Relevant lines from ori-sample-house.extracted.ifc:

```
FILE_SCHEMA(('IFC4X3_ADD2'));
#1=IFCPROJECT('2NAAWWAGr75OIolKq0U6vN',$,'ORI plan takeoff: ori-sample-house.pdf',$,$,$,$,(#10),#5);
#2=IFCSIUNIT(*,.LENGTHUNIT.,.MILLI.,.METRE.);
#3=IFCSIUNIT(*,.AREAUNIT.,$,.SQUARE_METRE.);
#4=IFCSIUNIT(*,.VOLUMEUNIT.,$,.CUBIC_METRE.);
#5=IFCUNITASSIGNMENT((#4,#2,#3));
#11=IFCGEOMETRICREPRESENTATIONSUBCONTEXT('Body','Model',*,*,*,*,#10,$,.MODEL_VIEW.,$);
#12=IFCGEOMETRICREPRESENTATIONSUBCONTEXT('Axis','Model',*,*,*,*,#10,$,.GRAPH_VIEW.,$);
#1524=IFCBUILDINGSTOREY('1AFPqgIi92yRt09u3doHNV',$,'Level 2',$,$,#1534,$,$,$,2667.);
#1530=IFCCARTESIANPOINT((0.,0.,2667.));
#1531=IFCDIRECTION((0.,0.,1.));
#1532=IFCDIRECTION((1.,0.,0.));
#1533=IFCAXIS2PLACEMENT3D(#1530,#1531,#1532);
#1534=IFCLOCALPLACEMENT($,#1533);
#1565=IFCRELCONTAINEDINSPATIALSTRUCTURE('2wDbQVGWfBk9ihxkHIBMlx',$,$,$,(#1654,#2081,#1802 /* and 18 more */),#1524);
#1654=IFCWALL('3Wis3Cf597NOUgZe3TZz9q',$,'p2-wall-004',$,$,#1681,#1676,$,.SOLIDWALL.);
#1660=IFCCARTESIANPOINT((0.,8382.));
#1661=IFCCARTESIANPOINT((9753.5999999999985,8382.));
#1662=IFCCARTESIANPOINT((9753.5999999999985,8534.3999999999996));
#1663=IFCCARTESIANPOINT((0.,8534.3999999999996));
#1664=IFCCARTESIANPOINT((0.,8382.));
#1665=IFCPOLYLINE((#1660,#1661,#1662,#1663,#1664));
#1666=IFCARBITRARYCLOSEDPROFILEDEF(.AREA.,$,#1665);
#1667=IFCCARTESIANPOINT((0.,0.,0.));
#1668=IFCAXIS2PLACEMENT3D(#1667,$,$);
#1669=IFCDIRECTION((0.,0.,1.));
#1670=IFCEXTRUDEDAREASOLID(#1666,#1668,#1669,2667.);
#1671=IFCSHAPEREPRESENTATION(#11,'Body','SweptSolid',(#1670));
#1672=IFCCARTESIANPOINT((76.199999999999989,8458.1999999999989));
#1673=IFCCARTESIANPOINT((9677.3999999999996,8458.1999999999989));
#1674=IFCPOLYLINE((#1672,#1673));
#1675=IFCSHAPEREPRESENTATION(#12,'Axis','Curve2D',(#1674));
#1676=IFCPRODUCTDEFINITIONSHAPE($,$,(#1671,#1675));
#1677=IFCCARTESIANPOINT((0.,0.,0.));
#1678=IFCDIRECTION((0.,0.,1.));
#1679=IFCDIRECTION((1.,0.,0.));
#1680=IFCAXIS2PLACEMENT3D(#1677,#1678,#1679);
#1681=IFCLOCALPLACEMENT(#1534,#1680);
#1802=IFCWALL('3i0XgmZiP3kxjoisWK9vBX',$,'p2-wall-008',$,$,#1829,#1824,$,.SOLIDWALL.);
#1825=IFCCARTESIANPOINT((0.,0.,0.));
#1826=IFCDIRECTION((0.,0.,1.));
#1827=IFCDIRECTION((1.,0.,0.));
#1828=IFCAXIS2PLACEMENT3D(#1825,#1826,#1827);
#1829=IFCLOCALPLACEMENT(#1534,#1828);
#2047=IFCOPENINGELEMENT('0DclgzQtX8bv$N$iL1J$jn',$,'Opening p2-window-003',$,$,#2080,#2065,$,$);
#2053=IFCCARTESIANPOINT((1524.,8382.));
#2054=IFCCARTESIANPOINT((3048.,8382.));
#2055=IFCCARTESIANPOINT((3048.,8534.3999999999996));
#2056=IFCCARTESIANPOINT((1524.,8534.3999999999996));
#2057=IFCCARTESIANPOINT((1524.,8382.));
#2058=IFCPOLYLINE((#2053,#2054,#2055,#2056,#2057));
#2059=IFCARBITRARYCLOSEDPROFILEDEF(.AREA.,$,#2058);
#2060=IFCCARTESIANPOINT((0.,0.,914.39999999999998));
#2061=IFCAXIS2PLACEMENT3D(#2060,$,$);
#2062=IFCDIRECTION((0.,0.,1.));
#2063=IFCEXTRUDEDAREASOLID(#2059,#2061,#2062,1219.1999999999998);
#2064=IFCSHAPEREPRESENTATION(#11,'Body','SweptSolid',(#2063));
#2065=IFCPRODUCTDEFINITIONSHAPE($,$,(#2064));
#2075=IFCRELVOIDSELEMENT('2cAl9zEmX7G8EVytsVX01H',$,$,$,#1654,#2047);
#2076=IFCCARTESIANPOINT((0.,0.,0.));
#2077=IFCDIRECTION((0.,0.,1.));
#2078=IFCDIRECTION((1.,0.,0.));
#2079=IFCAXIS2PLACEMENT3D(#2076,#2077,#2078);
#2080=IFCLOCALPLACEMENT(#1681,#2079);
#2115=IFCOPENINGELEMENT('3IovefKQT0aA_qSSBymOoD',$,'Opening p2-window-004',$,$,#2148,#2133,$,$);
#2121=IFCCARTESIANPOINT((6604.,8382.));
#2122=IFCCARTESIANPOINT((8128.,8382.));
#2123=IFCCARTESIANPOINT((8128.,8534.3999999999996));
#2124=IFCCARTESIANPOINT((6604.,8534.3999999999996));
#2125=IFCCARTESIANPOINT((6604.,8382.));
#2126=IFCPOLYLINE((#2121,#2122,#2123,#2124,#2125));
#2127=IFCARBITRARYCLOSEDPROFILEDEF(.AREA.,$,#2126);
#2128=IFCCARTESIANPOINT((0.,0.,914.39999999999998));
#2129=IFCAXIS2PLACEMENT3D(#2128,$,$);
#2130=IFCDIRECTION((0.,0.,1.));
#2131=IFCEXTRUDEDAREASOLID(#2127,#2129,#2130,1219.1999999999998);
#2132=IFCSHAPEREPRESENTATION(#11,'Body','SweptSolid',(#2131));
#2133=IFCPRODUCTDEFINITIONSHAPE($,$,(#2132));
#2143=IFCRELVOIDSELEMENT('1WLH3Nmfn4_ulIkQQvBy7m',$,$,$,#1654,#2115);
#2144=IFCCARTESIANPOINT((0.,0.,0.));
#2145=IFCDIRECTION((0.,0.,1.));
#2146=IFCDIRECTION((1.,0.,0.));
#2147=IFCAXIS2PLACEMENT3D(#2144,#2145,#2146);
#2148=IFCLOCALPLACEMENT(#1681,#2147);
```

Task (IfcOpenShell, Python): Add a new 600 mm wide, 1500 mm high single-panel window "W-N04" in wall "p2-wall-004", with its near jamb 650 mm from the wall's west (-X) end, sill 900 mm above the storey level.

```python
import numpy as np
import ifcopenshell
import ifcopenshell.api.feature
import ifcopenshell.api.geometry
import ifcopenshell.api.root
import ifcopenshell.api.spatial
import ifcopenshell.geom
import ifcopenshell.util.element
import ifcopenshell.util.placement
import ifcopenshell.util.representation
import ifcopenshell.util.shape
import ifcopenshell.util.unit

model = ifcopenshell.open("ori-sample-house.extracted.ifc")
unit_scale = ifcopenshell.util.unit.calculate_unit_scale(model)
settings = ifcopenshell.geom.settings()


def volume(element):
    """Net volume in cubic metres, openings subtracted."""
    shape = ifcopenshell.geom.create_shape(settings, element)
    return ifcopenshell.util.shape.get_volume(shape.geometry)


wall = model.by_guid("3Wis3Cf597NOUgZe3TZz9q")
storey = ifcopenshell.util.element.get_container(wall, ifc_class="IfcBuildingStorey")
context = ifcopenshell.util.representation.get_context(model, "Model", "Body", "MODEL_VIEW")
before = volume(wall)

width, height, from_end, sill = 0.6, 1.5, 0.65, 0.9  # metres

# The wall runs along its own X axis, and the end named is its -X end.
wall_shape = ifcopenshell.geom.create_shape(settings, wall)
x, y, z = ifcopenshell.util.shape.get_vertices(wall_shape.geometry).T
start = x.min() + from_end
face, thickness = float(y.min()), float(y.max() - y.min())
wall_matrix = ifcopenshell.util.placement.get_local_placement(wall.ObjectPlacement)
level = ifcopenshell.util.placement.get_local_placement(storey.ObjectPlacement)[2, 3]


def in_wall(x, y):
    """Placement at x, y metres in the wall's axes, at sill height."""
    matrix = wall_matrix.copy()
    matrix[:, 3] = wall_matrix @ np.array([x / unit_scale, y / unit_scale, 0.0, 1.0])
    matrix[2, 3] = level + sill / unit_scale
    return matrix


# Opening: a box that overshoots both wall faces by 50 mm.
opening = ifcopenshell.api.root.create_entity(model, ifc_class="IfcOpeningElement", predefined_type="OPENING")
box = ifcopenshell.api.geometry.add_wall_representation(
    model, context=context, length=width, height=height, thickness=thickness + 0.1
)
ifcopenshell.api.geometry.assign_representation(model, product=opening, representation=box)
ifcopenshell.api.geometry.edit_object_placement(model, product=opening, matrix=in_wall(start, face - 0.05), is_si=False)
ifcopenshell.api.feature.add_feature(model, feature=opening, element=wall)

window = ifcopenshell.api.root.create_entity(model, ifc_class="IfcWindow", name="W-N04", predefined_type="WINDOW")
window.OverallWidth, window.OverallHeight = width / unit_scale, height / unit_scale
window.PartitioningType = "SINGLE_PANEL"
body = ifcopenshell.api.geometry.add_window_representation(
    model,
    context=context,
    overall_width=window.OverallWidth,
    overall_height=window.OverallHeight,
    partition_type="SINGLE_PANEL",
)
ifcopenshell.api.geometry.assign_representation(model, product=window, representation=body)
ifcopenshell.api.spatial.assign_container(model, products=[window], relating_structure=storey)
ifcopenshell.api.feature.add_filling(model, opening=opening, element=window)

# Centre the window in the wall's thickness.
ifcopenshell.api.geometry.edit_object_placement(model, product=window, matrix=in_wall(start, face), is_si=False)
window_shape = ifcopenshell.geom.create_shape(settings, window)
depth = ifcopenshell.util.shape.get_vertices(window_shape.geometry)[:, 1]
offset = face + thickness / 2 - (depth.min() + depth.max()) / 2
ifcopenshell.api.geometry.edit_object_placement(model, product=window, matrix=in_wall(start, offset), is_si=False)

after = volume(wall)

print(f"wall volume {before:.3f} -> {after:.3f} m3")

model.write("ori-sample-house.extracted_v2.ifc")
```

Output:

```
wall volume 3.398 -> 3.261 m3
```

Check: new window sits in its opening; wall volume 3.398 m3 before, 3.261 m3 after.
